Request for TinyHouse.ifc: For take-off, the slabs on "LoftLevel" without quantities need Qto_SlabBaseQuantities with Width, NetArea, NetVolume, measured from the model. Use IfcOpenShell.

First a look at what the model holds.

```python
import ifcopenshell
import ifcopenshell.util.element
import ifcopenshell.util.unit

model = ifcopenshell.open("TinyHouse.ifc")
print(model.schema)
for unit_type in ("LENGTHUNIT", "AREAUNIT", "VOLUMEUNIT"):
    print(unit_type, ifcopenshell.util.unit.calculate_unit_scale(model, unit_type))
storey = next(s for s in model.by_type("IfcBuildingStorey") if s.Name == "LoftLevel")
slabs = [e for e in ifcopenshell.util.element.get_decomposition(storey) if e.is_a("IfcSlab")]
for e in sorted(slabs, key=lambda e: e.id()):
    print(e.id(), e.is_a(), e.Name, list(ifcopenshell.util.element.get_psets(e, qtos_only=True)), sep=" | ")
```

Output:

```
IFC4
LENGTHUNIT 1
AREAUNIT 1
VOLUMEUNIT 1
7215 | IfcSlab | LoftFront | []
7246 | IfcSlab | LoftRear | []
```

```python
import ifcopenshell
import ifcopenshell.api.pset
import ifcopenshell.geom
import ifcopenshell.util.element
import ifcopenshell.util.shape
import ifcopenshell.util.unit

model = ifcopenshell.open("TinyHouse.ifc")
unit_scale = ifcopenshell.util.unit.calculate_unit_scale(model)
area_scale = ifcopenshell.util.unit.calculate_unit_scale(model, "AREAUNIT")
volume_scale = ifcopenshell.util.unit.calculate_unit_scale(model, "VOLUMEUNIT")
settings = ifcopenshell.geom.settings()

storey = next(s for s in model.by_type("IfcBuildingStorey") if s.Name == "LoftLevel")
slabs = [e for e in ifcopenshell.util.element.get_decomposition(storey) if e.is_a("IfcSlab")]

for e in sorted(slabs, key=lambda e: e.id()):
    if ifcopenshell.util.element.get_psets(e, qtos_only=True, should_inherit=False):
        continue
    # Geometry comes back in metres, in the element's own axes.
    shape = ifcopenshell.geom.create_shape(settings, e)
    values = {
        "Width": ifcopenshell.util.shape.get_z(shape.geometry) / unit_scale,
        "NetArea": ifcopenshell.util.shape.get_footprint_area(shape.geometry) / area_scale,
        "NetVolume": ifcopenshell.util.shape.get_volume(shape.geometry) / volume_scale,
    }
    qto = ifcopenshell.api.pset.add_qto(model, product=e, name="Qto_SlabBaseQuantities")
    ifcopenshell.api.pset.edit_qto(model, qto=qto, properties=values)
    print(e.id(), {k: round(v, 3) for k, v in values.items()})

model.write("TinyHouse_rev.ifc")
```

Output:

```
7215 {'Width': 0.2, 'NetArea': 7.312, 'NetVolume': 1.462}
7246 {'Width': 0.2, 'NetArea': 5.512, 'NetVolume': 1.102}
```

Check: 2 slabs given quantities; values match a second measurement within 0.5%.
